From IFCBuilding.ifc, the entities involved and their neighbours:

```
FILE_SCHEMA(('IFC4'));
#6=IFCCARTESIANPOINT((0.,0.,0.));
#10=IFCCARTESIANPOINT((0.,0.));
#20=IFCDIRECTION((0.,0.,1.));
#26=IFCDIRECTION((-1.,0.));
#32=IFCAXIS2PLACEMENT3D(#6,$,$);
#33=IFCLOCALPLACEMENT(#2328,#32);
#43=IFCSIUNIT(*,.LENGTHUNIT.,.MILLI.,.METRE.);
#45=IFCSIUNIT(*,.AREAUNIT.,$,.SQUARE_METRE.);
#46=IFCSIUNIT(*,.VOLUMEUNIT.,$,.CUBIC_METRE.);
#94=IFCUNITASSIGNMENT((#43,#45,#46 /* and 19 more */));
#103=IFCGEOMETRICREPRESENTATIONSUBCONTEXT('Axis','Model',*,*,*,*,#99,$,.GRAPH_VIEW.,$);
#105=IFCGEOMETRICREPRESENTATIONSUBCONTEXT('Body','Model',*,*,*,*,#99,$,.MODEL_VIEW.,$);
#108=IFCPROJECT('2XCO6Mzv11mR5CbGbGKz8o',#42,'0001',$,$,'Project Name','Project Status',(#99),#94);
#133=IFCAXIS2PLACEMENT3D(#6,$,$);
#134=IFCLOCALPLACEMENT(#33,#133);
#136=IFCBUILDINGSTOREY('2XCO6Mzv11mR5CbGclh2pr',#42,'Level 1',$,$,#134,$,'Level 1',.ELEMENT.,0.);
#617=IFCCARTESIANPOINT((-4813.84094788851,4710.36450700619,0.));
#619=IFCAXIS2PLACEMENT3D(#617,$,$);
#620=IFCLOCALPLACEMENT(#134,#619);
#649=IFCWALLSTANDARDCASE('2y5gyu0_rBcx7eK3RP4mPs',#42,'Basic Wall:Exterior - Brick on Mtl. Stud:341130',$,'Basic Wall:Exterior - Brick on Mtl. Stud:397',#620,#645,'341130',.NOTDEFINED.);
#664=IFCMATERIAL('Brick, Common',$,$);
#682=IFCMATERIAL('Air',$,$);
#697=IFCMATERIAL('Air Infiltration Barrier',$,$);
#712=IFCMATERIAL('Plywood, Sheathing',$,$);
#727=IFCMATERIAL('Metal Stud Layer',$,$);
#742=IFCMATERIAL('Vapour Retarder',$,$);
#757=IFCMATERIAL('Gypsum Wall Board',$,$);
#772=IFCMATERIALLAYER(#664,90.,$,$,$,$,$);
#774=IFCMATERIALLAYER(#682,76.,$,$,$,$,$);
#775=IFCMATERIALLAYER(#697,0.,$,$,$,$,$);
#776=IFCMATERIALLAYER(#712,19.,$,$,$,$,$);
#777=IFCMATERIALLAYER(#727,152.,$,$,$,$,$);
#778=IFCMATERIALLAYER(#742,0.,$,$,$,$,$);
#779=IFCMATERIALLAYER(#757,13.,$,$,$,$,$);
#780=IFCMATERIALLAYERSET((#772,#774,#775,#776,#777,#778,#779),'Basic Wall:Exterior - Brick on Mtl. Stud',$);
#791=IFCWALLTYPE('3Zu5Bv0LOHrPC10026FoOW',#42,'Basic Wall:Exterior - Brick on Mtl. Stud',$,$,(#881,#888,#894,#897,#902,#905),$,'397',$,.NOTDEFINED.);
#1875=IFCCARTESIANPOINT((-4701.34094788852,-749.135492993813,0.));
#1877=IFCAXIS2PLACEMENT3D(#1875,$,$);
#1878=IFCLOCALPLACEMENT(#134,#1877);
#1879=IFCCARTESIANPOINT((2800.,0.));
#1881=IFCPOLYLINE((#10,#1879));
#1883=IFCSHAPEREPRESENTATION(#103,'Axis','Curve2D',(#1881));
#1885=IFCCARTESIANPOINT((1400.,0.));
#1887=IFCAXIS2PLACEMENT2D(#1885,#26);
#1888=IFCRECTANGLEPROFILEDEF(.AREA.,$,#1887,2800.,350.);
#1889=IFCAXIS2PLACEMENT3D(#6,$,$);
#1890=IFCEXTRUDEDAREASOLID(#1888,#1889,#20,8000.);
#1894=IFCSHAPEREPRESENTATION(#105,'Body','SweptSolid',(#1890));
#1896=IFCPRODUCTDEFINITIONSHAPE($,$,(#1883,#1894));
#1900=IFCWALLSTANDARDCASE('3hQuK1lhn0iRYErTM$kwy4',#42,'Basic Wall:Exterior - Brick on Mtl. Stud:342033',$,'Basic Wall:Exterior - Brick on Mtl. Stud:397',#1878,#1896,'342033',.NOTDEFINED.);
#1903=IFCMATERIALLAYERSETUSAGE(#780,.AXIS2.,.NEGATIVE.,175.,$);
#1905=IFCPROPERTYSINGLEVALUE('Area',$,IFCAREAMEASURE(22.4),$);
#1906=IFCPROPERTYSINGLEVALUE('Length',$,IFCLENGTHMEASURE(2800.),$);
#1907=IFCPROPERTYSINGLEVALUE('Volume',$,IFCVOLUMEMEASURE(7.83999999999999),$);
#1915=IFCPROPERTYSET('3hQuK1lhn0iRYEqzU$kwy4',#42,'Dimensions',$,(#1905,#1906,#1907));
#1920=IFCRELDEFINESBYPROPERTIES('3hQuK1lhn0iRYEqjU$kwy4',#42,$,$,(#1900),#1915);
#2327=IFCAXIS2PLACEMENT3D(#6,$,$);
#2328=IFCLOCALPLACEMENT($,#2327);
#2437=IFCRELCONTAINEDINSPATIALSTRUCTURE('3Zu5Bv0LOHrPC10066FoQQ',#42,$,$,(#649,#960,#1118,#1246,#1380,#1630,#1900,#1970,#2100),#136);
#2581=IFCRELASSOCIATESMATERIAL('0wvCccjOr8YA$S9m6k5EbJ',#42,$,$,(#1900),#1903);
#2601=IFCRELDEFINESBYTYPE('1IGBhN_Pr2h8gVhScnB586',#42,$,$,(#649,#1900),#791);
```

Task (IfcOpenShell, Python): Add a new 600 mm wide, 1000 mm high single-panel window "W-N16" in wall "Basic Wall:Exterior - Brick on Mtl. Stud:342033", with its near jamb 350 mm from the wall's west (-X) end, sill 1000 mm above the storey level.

```python
import numpy as np
import ifcopenshell
import ifcopenshell.api.feature
import ifcopenshell.api.geometry
import ifcopenshell.api.pset
import ifcopenshell.api.root
import ifcopenshell.api.spatial
import ifcopenshell.geom
import ifcopenshell.util.element
import ifcopenshell.util.placement
import ifcopenshell.util.representation
import ifcopenshell.util.shape
import ifcopenshell.util.unit

model = ifcopenshell.open("IFCBuilding.ifc")
unit_scale = ifcopenshell.util.unit.calculate_unit_scale(model)
area_scale = ifcopenshell.util.unit.calculate_unit_scale(model, "AREAUNIT")
volume_scale = ifcopenshell.util.unit.calculate_unit_scale(model, "VOLUMEUNIT")
settings = ifcopenshell.geom.settings()


def volume(element):
    """Net volume in cubic metres, openings subtracted."""
    shape = ifcopenshell.geom.create_shape(settings, element)
    return ifcopenshell.util.shape.get_volume(shape.geometry)


wall = model.by_guid("3hQuK1lhn0iRYErTM$kwy4")
storey = ifcopenshell.util.element.get_container(wall, ifc_class="IfcBuildingStorey")
context = ifcopenshell.util.representation.get_context(model, "Model", "Body", "MODEL_VIEW")
before = volume(wall)

width, height, from_end, sill = 0.6, 1, 0.35, 1  # metres

# The wall runs along its own X axis, and the end named is its -X end.
wall_shape = ifcopenshell.geom.create_shape(settings, wall)
x, y, z = ifcopenshell.util.shape.get_vertices(wall_shape.geometry).T
start = x.min() + from_end
face, thickness = float(y.min()), float(y.max() - y.min())
wall_matrix = ifcopenshell.util.placement.get_local_placement(wall.ObjectPlacement)
level = ifcopenshell.util.placement.get_local_placement(storey.ObjectPlacement)[2, 3]


def in_wall(x, y):
    """Placement at x, y metres in the wall's axes, at sill height."""
    matrix = wall_matrix.copy()
    matrix[:, 3] = wall_matrix @ np.array([x / unit_scale, y / unit_scale, 0.0, 1.0])
    matrix[2, 3] = level + sill / unit_scale
    return matrix


# Opening: a box that overshoots both wall faces by 50 mm.
opening = ifcopenshell.api.root.create_entity(model, ifc_class="IfcOpeningElement", predefined_type="OPENING")
box = ifcopenshell.api.geometry.add_wall_representation(
    model, context=context, length=width, height=height, thickness=thickness + 0.1
)
ifcopenshell.api.geometry.assign_representation(model, product=opening, representation=box)
ifcopenshell.api.geometry.edit_object_placement(model, product=opening, matrix=in_wall(start, face - 0.05), is_si=False)
ifcopenshell.api.feature.add_feature(model, feature=opening, element=wall)

window = ifcopenshell.api.root.create_entity(model, ifc_class="IfcWindow", name="W-N16", predefined_type="WINDOW")
window.OverallWidth, window.OverallHeight = width / unit_scale, height / unit_scale
window.PartitioningType = "SINGLE_PANEL"
body = ifcopenshell.api.geometry.add_window_representation(
    model,
    context=context,
    overall_width=window.OverallWidth,
    overall_height=window.OverallHeight,
    partition_type="SINGLE_PANEL",
)
ifcopenshell.api.geometry.assign_representation(model, product=window, representation=body)
ifcopenshell.api.spatial.assign_container(model, products=[window], relating_structure=storey)
ifcopenshell.api.feature.add_filling(model, opening=opening, element=window)

# Centre the window in the wall's thickness.
ifcopenshell.api.geometry.edit_object_placement(model, product=window, matrix=in_wall(start, face), is_si=False)
window_shape = ifcopenshell.geom.create_shape(settings, window)
depth = ifcopenshell.util.shape.get_vertices(window_shape.geometry)[:, 1]
offset = face + thickness / 2 - (depth.min() + depth.max()) / 2
ifcopenshell.api.geometry.edit_object_placement(model, product=window, matrix=in_wall(start, offset), is_si=False)

after = volume(wall)

# Update the wall's stored quantities.
pset = model.by_id(ifcopenshell.util.element.get_pset(wall, "Dimensions", should_inherit=False)["id"])
ifcopenshell.api.pset.edit_pset(model, pset=pset, properties={
    "Area": model.create_entity("IfcAreaMeasure", after / thickness / area_scale),
    "Volume": model.create_entity("IfcVolumeMeasure", after / volume_scale),
})

print(f"wall volume {before:.3f} -> {after:.3f} m3")

model.write("IFCBuilding-out.ifc")
```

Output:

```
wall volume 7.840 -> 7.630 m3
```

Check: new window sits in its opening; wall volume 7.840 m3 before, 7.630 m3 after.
